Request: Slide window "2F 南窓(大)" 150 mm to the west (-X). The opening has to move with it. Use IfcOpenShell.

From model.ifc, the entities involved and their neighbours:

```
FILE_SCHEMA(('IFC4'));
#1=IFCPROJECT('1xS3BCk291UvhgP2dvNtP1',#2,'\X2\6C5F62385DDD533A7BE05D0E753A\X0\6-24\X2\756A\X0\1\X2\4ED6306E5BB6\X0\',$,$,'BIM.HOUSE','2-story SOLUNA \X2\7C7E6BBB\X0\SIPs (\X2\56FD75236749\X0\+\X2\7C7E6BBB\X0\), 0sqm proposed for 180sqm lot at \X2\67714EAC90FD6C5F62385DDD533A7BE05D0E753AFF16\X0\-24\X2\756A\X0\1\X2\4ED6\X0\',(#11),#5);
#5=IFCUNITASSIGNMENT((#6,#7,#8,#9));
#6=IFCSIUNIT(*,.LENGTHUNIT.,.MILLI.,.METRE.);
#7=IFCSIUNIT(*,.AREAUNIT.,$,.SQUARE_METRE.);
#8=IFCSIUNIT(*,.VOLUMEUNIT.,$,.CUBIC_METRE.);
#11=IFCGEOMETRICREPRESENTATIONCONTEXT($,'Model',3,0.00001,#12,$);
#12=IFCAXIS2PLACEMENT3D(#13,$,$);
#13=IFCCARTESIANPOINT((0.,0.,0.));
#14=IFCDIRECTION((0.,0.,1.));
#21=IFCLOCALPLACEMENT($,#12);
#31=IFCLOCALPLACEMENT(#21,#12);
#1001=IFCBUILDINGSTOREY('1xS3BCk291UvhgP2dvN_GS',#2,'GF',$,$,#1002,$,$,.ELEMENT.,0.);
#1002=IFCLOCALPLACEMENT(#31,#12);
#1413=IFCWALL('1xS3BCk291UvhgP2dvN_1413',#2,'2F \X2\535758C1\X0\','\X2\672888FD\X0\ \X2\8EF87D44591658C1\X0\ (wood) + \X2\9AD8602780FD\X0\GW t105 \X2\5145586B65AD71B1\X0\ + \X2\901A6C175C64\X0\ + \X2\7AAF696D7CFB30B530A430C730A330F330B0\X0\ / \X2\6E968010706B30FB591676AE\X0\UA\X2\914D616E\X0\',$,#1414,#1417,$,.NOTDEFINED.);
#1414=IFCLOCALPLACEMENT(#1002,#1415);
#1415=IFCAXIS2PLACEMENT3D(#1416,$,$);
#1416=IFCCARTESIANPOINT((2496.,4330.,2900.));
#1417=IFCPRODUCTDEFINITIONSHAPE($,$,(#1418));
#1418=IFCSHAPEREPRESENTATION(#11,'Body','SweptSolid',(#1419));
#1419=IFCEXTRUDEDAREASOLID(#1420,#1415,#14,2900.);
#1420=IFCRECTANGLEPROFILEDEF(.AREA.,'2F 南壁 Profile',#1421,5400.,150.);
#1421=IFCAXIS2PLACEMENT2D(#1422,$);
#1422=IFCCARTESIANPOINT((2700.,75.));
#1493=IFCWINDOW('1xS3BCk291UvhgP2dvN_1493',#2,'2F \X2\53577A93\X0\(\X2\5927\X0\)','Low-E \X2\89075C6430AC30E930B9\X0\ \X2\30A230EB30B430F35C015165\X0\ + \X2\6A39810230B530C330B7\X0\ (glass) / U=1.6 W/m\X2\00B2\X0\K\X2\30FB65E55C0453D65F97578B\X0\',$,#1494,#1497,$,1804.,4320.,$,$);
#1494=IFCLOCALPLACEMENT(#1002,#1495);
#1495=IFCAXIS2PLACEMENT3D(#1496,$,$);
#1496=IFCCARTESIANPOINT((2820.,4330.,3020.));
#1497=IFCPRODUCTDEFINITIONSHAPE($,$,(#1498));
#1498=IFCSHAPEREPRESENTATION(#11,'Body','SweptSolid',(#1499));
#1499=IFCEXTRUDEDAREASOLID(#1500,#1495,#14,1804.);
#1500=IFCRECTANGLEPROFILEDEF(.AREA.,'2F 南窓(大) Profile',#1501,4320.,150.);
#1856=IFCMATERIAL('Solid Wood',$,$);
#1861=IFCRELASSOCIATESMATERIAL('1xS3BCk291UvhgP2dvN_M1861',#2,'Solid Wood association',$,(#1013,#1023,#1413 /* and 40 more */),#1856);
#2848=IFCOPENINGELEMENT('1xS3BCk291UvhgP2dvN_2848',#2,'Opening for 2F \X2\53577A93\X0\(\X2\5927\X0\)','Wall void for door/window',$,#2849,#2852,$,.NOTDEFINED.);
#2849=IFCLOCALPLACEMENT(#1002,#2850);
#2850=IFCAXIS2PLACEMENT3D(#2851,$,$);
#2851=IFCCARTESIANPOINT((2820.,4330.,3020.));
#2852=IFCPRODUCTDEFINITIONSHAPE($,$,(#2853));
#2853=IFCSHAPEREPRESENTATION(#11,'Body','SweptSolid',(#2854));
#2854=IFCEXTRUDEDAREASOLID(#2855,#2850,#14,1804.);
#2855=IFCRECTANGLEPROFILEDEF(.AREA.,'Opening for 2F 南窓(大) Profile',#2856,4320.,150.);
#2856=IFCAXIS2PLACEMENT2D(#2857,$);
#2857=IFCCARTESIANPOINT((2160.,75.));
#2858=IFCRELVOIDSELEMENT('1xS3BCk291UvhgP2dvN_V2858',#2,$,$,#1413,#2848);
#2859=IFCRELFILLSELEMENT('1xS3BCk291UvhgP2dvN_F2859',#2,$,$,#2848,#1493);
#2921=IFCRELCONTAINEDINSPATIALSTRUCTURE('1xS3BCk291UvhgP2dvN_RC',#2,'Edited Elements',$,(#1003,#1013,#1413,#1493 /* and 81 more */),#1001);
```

```python
import ifcopenshell
import ifcopenshell.api.geometry
import ifcopenshell.util.placement
import ifcopenshell.util.unit

model = ifcopenshell.open("model.ifc")
unit_scale = ifcopenshell.util.unit.calculate_unit_scale(model)

window = model.by_guid("1xS3BCk291UvhgP2dvN_1493")
opening = window.FillsVoids[0].RelatingOpeningElement
wall = opening.VoidsElements[0].RelatingBuildingElement

wall_matrix = ifcopenshell.util.placement.get_local_placement(wall.ObjectPlacement)
shift = wall_matrix[:3, 0] * -0.15 / unit_scale
before = ifcopenshell.util.placement.get_local_placement(window.ObjectPlacement)[:3, 3].copy()

# The window is not placed relative to its opening, so move both.
for product in (opening, window):
    matrix = ifcopenshell.util.placement.get_local_placement(product.ObjectPlacement)
    matrix[:3, 3] += shift
    ifcopenshell.api.geometry.edit_object_placement(model, product=product, matrix=matrix, is_si=False)

after = ifcopenshell.util.placement.get_local_placement(window.ObjectPlacement)[:3, 3]
print("window moved by", (after - before).round(3) + 0.0)

model.write("model_rev.ifc")
```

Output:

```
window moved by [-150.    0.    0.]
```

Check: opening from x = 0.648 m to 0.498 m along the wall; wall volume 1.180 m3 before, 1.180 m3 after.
